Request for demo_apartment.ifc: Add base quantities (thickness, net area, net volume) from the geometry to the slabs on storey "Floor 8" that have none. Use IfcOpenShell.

First a look at what the model holds.

```python
import ifcopenshell
import ifcopenshell.util.element
import ifcopenshell.util.unit

model = ifcopenshell.open("demo_apartment.ifc")
print(model.schema)
for unit_type in ("LENGTHUNIT", "AREAUNIT", "VOLUMEUNIT"):
    print(unit_type, ifcopenshell.util.unit.calculate_unit_scale(model, unit_type))
storey = next(s for s in model.by_type("IfcBuildingStorey") if s.Name == "Floor 8")
slabs = [e for e in ifcopenshell.util.element.get_decomposition(storey) if e.is_a("IfcSlab")]
for e in sorted(slabs, key=lambda e: e.id()):
    print(e.id(), e.is_a(), e.Name, list(ifcopenshell.util.element.get_psets(e, qtos_only=True)), sep=" | ")
```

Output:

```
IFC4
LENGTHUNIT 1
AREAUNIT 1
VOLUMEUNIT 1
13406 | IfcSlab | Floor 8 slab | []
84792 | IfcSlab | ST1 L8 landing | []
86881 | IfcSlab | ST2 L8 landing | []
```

```python
import ifcopenshell
import ifcopenshell.api.pset
import ifcopenshell.geom
import ifcopenshell.util.element
import ifcopenshell.util.shape
import ifcopenshell.util.unit

model = ifcopenshell.open("demo_apartment.ifc")
unit_scale = ifcopenshell.util.unit.calculate_unit_scale(model)
area_scale = ifcopenshell.util.unit.calculate_unit_scale(model, "AREAUNIT")
volume_scale = ifcopenshell.util.unit.calculate_unit_scale(model, "VOLUMEUNIT")
settings = ifcopenshell.geom.settings()

storey = next(s for s in model.by_type("IfcBuildingStorey") if s.Name == "Floor 8")
slabs = [e for e in ifcopenshell.util.element.get_decomposition(storey) if e.is_a("IfcSlab")]

for e in sorted(slabs, key=lambda e: e.id()):
    if ifcopenshell.util.element.get_psets(e, qtos_only=True, should_inherit=False):
        continue
    # Geometry comes back in metres, in the element's own axes.
    shape = ifcopenshell.geom.create_shape(settings, e)
    values = {
        "Width": ifcopenshell.util.shape.get_z(shape.geometry) / unit_scale,
        "NetArea": ifcopenshell.util.shape.get_footprint_area(shape.geometry) / area_scale,
        "NetVolume": ifcopenshell.util.shape.get_volume(shape.geometry) / volume_scale,
    }
    qto = ifcopenshell.api.pset.add_qto(model, product=e, name="Qto_SlabBaseQuantities")
    ifcopenshell.api.pset.edit_qto(model, qto=qto, properties=values)
    print(e.id(), {k: round(v, 3) for k, v in values.items()})

model.write("demo_apartment-out.ifc")
```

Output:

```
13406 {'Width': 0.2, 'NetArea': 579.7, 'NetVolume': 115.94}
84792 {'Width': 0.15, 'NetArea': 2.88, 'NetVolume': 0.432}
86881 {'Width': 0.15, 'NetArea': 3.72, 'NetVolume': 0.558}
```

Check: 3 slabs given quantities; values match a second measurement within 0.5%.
